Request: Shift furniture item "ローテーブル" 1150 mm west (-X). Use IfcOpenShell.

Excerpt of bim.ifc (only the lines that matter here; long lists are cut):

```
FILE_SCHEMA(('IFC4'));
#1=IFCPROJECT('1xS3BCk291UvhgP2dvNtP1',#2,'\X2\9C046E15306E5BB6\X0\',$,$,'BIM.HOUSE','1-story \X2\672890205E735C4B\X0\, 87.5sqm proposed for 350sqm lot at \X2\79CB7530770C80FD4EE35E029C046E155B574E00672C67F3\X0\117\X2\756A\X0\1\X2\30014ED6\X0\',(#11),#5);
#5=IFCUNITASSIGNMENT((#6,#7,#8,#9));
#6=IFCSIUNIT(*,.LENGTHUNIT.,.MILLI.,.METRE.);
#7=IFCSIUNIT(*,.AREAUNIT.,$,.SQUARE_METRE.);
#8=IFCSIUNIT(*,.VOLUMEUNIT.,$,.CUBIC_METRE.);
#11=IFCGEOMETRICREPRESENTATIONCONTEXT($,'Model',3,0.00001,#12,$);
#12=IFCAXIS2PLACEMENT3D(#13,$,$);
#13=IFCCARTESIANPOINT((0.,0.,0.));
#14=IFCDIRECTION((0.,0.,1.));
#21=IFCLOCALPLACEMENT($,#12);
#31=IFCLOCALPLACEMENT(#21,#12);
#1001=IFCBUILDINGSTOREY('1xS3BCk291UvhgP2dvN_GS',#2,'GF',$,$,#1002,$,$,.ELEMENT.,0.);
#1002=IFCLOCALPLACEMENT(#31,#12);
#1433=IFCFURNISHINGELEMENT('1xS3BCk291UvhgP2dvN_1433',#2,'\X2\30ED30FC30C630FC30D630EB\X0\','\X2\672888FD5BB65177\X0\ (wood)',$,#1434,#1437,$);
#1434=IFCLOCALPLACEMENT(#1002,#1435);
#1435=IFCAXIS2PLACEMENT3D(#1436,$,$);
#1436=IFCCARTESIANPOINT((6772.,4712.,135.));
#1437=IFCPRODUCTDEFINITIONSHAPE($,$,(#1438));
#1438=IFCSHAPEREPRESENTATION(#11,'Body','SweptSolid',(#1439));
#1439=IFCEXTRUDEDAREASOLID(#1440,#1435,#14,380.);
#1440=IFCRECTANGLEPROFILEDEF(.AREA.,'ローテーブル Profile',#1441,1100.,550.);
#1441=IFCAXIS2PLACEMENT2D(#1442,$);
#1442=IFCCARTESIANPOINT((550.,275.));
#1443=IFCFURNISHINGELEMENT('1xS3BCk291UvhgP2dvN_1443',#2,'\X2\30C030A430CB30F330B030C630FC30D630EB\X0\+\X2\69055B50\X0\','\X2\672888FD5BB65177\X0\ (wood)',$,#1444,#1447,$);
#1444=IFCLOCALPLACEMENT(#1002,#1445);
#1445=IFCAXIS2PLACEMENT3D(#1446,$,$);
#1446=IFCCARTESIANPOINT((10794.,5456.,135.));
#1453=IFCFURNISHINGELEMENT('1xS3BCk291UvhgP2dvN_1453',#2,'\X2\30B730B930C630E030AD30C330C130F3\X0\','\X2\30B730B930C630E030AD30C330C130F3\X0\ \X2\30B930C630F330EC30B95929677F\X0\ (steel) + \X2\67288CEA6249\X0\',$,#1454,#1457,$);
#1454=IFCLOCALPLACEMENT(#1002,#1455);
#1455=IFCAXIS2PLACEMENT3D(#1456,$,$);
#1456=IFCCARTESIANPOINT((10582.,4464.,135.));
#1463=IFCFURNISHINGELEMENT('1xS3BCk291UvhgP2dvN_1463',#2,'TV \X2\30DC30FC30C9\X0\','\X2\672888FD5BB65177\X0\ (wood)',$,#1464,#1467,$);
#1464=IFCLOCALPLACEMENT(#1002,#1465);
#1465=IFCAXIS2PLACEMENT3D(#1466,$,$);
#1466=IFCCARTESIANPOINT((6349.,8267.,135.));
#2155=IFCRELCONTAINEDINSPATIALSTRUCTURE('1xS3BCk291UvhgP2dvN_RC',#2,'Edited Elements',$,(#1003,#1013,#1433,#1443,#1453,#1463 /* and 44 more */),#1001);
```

```python
import ifcopenshell
import ifcopenshell.api.geometry
import ifcopenshell.util.placement
import ifcopenshell.util.unit

model = ifcopenshell.open("bim.ifc")
unit_scale = ifcopenshell.util.unit.calculate_unit_scale(model)

item = model.by_guid("1xS3BCk291UvhgP2dvN_1433")
matrix = ifcopenshell.util.placement.get_local_placement(item.ObjectPlacement)
matrix[0, 3] -= 1.15 / unit_scale
ifcopenshell.api.geometry.edit_object_placement(model, product=item, matrix=matrix, is_si=False)

print(ifcopenshell.util.placement.get_local_placement(item.ObjectPlacement).round(3) + 0.0)

model.write("bim_rev.ifc")
```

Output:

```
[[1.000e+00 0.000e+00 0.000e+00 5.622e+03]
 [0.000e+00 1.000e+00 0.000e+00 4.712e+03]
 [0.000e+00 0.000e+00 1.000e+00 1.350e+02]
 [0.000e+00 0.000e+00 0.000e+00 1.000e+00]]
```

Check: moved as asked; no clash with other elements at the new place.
